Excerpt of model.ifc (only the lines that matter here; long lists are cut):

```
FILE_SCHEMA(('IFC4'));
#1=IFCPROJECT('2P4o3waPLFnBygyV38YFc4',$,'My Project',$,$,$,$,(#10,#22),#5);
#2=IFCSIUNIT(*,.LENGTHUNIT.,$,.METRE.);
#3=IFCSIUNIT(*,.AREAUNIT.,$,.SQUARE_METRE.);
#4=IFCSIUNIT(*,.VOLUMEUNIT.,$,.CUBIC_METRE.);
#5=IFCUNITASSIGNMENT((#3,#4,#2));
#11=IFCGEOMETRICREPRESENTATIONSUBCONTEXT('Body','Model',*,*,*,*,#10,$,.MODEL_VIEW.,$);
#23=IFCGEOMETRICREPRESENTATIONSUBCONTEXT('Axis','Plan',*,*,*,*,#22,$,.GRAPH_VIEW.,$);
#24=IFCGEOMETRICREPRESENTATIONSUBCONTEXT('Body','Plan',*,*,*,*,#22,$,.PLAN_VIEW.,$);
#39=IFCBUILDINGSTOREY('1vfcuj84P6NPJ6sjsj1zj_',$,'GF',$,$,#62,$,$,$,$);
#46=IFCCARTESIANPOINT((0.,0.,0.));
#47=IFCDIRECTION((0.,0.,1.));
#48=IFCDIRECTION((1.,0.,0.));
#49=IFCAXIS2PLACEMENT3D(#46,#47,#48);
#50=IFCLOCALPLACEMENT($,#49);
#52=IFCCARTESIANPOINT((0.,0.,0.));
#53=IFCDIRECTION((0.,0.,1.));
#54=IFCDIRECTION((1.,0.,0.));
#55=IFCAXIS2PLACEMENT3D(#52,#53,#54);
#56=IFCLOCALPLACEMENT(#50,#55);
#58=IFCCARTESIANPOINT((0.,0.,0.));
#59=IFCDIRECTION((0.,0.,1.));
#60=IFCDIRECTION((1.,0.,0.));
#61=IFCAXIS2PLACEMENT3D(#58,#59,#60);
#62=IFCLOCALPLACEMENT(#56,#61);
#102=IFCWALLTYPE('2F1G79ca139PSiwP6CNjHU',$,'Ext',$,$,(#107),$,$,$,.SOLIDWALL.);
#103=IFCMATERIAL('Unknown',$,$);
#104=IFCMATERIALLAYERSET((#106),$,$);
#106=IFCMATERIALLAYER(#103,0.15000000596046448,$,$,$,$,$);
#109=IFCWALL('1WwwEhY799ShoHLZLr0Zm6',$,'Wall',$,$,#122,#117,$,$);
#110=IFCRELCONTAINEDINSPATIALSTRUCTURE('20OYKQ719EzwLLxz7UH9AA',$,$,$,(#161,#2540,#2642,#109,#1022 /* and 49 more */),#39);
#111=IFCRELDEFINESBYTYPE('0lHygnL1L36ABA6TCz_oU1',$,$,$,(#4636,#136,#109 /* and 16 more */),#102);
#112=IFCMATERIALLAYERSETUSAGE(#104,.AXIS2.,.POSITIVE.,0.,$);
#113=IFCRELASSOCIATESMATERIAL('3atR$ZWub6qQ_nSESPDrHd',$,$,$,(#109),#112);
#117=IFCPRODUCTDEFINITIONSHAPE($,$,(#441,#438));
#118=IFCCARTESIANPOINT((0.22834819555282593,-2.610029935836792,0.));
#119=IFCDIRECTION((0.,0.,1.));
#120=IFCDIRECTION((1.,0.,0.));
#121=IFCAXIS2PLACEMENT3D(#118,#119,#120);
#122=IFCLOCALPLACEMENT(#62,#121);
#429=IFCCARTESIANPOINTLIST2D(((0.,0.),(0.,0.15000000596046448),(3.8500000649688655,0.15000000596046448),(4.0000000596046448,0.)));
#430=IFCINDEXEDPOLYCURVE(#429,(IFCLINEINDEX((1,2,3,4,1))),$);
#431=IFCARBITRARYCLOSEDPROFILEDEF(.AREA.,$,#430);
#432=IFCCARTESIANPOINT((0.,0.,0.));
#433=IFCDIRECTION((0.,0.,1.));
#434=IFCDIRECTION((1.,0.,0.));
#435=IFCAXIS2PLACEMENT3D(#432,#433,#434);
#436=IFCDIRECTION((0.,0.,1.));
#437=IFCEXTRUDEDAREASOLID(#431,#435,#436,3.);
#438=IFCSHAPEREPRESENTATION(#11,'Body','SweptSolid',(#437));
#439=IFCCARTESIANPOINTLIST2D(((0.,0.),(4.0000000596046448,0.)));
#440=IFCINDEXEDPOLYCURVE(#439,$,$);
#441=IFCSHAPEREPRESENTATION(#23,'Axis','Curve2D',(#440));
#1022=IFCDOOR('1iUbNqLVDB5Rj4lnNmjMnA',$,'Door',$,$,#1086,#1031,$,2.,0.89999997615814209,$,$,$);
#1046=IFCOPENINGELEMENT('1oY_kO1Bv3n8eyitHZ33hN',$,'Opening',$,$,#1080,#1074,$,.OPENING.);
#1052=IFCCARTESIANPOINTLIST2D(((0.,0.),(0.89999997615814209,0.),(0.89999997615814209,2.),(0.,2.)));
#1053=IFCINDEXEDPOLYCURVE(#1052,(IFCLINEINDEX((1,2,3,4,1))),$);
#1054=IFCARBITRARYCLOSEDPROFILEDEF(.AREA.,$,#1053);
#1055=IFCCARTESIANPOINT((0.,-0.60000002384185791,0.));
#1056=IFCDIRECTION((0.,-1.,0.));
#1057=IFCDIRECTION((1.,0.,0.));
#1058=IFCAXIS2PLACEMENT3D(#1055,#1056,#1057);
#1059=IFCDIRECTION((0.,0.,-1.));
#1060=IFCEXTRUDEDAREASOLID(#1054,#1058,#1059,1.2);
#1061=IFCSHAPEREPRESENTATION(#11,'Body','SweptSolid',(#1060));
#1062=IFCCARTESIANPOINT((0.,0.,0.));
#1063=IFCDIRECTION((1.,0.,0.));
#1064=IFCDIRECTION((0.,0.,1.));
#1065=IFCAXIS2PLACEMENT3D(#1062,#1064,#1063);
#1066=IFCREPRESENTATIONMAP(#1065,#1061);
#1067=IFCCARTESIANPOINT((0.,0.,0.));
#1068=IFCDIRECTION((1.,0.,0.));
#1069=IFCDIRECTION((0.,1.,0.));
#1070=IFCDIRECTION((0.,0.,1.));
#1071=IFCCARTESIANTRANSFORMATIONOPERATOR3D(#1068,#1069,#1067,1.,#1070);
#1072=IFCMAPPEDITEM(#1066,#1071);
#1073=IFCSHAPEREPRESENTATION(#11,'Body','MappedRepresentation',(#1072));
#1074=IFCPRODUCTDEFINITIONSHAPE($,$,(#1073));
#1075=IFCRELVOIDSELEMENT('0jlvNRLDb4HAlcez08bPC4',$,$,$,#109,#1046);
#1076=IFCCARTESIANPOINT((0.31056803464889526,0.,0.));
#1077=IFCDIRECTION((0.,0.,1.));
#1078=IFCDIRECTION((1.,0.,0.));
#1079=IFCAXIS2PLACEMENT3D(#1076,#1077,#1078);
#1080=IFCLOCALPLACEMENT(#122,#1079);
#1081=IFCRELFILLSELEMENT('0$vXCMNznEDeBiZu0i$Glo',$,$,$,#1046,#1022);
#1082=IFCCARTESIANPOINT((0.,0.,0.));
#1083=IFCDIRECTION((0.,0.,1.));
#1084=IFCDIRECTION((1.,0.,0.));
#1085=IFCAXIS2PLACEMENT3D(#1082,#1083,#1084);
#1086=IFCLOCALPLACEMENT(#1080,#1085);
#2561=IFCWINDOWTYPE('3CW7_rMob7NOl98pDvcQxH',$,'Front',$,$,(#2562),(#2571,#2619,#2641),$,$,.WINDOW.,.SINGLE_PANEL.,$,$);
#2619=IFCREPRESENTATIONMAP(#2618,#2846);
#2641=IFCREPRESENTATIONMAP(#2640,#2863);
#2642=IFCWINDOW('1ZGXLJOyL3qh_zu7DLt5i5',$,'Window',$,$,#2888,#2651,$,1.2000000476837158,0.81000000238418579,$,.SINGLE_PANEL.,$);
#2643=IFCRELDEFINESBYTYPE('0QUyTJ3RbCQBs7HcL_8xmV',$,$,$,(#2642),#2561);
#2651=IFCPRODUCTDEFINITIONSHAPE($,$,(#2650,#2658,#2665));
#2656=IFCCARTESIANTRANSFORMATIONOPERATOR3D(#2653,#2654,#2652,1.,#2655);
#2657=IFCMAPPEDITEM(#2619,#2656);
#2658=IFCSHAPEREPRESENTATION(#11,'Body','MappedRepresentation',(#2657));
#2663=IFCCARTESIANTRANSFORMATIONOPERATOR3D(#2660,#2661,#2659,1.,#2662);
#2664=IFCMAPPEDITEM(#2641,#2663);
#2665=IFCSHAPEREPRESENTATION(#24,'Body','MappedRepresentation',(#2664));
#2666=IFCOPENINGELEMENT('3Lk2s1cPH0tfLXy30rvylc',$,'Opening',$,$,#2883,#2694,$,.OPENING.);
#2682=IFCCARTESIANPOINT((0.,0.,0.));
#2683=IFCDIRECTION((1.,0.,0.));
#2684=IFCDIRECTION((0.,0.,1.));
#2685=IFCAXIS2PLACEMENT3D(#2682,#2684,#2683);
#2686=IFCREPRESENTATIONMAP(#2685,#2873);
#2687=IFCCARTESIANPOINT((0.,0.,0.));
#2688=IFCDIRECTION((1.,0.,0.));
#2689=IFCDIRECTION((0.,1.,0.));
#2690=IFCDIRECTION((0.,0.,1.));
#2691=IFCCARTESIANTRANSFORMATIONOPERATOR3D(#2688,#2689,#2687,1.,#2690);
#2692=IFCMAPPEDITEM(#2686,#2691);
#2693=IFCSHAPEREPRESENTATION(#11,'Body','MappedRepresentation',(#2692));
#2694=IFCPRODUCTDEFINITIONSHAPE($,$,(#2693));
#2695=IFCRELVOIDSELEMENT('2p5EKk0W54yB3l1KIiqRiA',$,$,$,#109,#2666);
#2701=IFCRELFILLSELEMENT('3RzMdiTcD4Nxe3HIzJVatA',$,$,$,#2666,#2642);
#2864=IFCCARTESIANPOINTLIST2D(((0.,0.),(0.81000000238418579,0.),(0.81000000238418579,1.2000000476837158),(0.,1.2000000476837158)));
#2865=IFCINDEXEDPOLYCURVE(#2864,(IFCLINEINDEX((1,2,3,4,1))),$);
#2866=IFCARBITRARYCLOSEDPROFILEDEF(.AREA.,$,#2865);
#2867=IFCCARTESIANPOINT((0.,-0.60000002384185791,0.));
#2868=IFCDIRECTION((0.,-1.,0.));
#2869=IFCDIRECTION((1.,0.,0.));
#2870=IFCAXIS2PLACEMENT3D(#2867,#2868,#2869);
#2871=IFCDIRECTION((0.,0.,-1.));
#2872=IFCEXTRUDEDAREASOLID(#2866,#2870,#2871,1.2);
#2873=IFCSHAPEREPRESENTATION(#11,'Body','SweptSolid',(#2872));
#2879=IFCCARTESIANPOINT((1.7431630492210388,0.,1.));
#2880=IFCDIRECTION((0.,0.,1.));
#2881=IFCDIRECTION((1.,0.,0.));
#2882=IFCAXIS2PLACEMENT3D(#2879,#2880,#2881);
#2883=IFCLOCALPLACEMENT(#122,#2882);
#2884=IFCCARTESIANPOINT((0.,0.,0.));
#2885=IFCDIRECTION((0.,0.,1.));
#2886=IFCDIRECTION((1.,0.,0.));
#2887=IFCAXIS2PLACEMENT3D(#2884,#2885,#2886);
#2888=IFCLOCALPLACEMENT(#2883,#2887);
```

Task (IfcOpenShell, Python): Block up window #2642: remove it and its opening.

```python
import ifcopenshell
import ifcopenshell.api.feature
import ifcopenshell.api.root
import ifcopenshell.geom
import ifcopenshell.util.shape

model = ifcopenshell.open("model.ifc")
settings = ifcopenshell.geom.settings()


def volume(element):
    """Net volume in cubic metres, openings subtracted."""
    shape = ifcopenshell.geom.create_shape(settings, element)
    return ifcopenshell.util.shape.get_volume(shape.geometry)


window = model.by_guid("1ZGXLJOyL3qh_zu7DLt5i5")
opening = window.FillsVoids[0].RelatingOpeningElement
wall = opening.VoidsElements[0].RelatingBuildingElement
before = volume(wall)

ifcopenshell.api.root.remove_product(model, product=window)
ifcopenshell.api.feature.remove_feature(model, feature=opening)

after = volume(wall)

print(f"wall volume {before:.3f} -> {after:.3f} m3")

model.write("model-out.ifc")
```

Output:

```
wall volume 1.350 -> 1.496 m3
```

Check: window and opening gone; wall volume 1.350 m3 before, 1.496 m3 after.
